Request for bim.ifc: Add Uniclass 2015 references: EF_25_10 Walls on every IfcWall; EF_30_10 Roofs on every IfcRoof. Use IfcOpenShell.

First a look at what the model holds.

```python
import ifcopenshell

model = ifcopenshell.open("bim.ifc")
print(model.schema)
print("classifications:", [c.Name for c in model.by_type("IfcClassification")])
for ifc_class in ("IfcDoor", "IfcRoof", "IfcStair", "IfcWall", "IfcWindow"):
    print(ifc_class, len(model.by_type(ifc_class)))
```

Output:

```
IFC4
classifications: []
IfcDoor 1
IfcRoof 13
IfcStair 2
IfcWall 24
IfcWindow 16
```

```python
import ifcopenshell
import ifcopenshell.api.classification

model = ifcopenshell.open("bim.ifc")

system = ifcopenshell.api.classification.add_classification(model, classification="Uniclass 2015")

codes = {
    "IfcWall": ("EF_25_10", "Walls"),
    "IfcRoof": ("EF_30_10", "Roofs"),
}
for ifc_class, (code, name) in codes.items():
    products = model.by_type(ifc_class)
    ifcopenshell.api.classification.add_reference(
        model, products=products, classification=system, identification=code, name=name
    )
    print(code, len(products))

model.write("bim_rev.ifc")
```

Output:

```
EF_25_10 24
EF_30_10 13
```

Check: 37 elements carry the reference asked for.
